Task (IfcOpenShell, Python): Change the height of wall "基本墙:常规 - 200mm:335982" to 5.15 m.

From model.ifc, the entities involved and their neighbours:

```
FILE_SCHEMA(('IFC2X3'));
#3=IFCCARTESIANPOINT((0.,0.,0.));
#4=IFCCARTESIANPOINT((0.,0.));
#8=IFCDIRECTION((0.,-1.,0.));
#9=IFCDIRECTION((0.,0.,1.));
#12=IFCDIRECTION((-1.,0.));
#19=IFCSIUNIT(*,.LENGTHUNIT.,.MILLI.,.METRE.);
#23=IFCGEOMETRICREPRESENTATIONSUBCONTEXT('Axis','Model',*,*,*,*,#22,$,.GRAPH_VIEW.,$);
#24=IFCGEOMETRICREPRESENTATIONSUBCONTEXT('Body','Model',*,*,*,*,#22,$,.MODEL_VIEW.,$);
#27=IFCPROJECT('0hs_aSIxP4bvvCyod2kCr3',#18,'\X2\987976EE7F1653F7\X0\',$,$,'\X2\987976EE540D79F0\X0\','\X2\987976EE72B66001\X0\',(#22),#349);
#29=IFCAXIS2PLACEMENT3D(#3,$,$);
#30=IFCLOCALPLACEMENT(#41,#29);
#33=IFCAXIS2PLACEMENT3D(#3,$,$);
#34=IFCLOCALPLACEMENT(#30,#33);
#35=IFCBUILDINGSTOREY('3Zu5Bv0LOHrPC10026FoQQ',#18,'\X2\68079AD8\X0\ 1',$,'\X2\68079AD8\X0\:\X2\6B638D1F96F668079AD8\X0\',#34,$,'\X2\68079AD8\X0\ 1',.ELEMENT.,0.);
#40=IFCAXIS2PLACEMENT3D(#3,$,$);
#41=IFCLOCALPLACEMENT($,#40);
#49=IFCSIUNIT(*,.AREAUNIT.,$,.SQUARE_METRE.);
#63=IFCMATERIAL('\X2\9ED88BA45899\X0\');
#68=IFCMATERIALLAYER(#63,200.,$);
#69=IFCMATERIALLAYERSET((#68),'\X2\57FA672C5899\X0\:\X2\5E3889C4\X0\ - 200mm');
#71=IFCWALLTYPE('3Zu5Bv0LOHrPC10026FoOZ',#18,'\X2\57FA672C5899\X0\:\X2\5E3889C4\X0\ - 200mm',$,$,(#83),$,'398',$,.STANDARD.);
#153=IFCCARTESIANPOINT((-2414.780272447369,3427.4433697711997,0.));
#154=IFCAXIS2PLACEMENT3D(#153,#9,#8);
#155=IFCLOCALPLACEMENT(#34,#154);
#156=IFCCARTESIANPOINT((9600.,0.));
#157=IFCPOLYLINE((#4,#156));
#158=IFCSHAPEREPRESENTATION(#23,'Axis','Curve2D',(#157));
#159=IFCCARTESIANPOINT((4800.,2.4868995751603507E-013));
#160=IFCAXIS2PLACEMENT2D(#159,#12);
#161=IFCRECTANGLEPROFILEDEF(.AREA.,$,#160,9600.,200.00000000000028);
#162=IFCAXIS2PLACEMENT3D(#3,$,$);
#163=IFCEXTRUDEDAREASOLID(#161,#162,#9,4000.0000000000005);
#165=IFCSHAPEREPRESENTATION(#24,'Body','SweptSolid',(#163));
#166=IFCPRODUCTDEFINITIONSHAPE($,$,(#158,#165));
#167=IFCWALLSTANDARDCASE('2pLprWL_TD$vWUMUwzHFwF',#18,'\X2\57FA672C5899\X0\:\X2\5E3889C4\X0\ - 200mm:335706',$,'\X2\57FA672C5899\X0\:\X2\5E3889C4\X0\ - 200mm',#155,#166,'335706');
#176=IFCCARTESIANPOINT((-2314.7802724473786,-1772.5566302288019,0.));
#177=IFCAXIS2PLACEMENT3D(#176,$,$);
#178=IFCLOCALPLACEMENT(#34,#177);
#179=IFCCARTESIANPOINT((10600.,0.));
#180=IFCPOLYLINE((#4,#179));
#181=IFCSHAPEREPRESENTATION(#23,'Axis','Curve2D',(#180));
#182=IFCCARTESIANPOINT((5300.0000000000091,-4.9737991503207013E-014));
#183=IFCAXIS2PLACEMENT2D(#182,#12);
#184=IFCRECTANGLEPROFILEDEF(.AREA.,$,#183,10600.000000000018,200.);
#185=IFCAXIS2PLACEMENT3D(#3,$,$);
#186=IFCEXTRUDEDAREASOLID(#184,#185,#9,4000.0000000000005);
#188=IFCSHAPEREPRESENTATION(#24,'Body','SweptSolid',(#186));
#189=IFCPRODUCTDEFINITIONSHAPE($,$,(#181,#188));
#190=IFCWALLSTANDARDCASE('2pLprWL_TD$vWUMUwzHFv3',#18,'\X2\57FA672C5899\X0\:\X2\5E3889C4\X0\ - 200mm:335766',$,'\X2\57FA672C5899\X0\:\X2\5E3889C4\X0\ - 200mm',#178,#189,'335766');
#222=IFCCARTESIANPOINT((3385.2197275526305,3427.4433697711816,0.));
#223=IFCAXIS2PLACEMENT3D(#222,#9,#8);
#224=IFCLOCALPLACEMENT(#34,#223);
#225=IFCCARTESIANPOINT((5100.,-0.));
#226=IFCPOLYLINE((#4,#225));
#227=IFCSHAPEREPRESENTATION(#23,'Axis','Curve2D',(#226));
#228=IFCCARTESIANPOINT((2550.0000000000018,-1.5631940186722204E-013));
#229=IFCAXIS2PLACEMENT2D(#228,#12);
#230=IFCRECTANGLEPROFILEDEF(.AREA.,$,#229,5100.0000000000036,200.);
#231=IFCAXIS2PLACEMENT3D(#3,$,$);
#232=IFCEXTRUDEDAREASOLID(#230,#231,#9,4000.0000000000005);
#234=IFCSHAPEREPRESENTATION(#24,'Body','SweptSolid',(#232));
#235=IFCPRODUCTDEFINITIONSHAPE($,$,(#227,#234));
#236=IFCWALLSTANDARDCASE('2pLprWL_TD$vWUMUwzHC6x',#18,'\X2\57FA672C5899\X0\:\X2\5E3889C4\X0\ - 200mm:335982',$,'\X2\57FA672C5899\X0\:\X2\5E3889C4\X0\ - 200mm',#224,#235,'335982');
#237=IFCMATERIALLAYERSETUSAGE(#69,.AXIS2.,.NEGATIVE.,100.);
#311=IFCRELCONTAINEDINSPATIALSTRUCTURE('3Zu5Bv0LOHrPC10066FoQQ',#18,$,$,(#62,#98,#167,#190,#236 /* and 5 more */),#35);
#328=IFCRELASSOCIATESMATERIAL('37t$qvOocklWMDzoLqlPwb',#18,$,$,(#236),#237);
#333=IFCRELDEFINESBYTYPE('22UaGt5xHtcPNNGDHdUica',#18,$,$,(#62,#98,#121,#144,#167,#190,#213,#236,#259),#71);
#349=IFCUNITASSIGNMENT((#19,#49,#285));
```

```python
import ifcopenshell
import ifcopenshell.geom
import ifcopenshell.util.representation
import ifcopenshell.util.shape
import ifcopenshell.util.unit

model = ifcopenshell.open("model.ifc")
unit_scale = ifcopenshell.util.unit.calculate_unit_scale(model)
settings = ifcopenshell.geom.settings()


def volume(element):
    """Net volume in cubic metres, openings subtracted."""
    shape = ifcopenshell.geom.create_shape(settings, element)
    return ifcopenshell.util.shape.get_volume(shape.geometry)


wall = model.by_id(236)
before = volume(wall)

body = ifcopenshell.util.representation.get_representation(wall, "Model", "Body")
solid = body.Items[0]
old_height = solid.Depth
solid.Depth = 5.15 / unit_scale
after = volume(wall)

print(f"height {old_height:g} -> {solid.Depth:g}, volume {before:.3f} -> {after:.3f} m3")

model.write("model_rev.ifc")
```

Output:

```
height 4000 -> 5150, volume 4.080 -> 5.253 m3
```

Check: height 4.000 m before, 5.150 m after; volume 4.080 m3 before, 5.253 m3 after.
